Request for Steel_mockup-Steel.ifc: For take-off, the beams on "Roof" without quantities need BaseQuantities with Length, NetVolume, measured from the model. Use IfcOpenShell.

First a look at what the model holds.

```python
import ifcopenshell
import ifcopenshell.util.element
import ifcopenshell.util.unit

model = ifcopenshell.open("Steel_mockup-Steel.ifc")
print(model.schema)
for unit_type in ("LENGTHUNIT", "AREAUNIT", "VOLUMEUNIT"):
    print(unit_type, ifcopenshell.util.unit.calculate_unit_scale(model, unit_type))
storey = next(s for s in model.by_type("IfcBuildingStorey") if s.Name == "Roof")
beams = [e for e in ifcopenshell.util.element.get_decomposition(storey) if e.is_a("IfcBeam")]
for e in sorted(beams, key=lambda e: e.id()):
    print(e.id(), e.is_a(), e.Name, list(ifcopenshell.util.element.get_psets(e, qtos_only=True)), sep=" | ")
```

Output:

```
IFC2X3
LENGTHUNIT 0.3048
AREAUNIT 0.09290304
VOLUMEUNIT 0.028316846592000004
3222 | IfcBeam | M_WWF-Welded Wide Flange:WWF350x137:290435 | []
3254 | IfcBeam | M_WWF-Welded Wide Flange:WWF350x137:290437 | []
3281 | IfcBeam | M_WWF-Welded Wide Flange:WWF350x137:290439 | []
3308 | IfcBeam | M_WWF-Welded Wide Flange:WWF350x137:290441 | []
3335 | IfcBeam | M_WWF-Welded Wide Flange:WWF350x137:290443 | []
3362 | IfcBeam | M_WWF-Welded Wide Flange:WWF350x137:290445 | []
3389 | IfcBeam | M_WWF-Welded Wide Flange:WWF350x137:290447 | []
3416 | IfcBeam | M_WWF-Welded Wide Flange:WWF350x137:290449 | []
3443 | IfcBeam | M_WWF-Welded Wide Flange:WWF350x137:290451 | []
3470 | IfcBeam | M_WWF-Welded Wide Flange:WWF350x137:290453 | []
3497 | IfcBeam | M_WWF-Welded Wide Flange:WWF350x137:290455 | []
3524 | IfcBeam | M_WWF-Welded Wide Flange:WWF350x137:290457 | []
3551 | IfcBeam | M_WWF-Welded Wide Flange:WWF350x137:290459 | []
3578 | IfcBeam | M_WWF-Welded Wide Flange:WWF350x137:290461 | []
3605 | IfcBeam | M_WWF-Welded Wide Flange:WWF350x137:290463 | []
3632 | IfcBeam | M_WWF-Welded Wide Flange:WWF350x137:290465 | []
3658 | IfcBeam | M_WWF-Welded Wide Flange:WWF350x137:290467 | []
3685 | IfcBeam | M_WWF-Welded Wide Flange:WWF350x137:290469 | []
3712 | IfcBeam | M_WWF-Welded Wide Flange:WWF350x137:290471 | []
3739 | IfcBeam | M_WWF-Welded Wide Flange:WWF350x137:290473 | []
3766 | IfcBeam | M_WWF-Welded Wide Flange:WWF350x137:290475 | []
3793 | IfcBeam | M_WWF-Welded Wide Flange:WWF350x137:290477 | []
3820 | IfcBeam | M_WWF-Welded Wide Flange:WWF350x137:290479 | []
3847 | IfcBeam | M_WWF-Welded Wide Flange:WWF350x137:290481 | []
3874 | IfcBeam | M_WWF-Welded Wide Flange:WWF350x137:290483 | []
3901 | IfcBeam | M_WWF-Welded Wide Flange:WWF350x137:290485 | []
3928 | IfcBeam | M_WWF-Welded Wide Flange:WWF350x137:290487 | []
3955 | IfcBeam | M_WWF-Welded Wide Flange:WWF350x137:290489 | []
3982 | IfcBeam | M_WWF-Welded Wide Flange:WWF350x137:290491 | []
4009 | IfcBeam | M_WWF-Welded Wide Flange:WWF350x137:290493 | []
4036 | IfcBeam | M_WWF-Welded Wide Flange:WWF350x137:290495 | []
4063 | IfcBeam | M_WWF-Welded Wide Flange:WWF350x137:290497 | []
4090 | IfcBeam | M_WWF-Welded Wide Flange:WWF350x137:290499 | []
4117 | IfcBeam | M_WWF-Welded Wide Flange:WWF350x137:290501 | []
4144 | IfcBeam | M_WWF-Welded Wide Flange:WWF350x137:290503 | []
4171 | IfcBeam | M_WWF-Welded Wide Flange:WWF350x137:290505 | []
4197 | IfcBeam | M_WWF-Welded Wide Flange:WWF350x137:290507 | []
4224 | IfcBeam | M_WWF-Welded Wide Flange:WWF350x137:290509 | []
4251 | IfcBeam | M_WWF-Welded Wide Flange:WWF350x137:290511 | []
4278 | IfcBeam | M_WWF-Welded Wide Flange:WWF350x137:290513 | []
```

```python
import ifcopenshell
import ifcopenshell.api.pset
import ifcopenshell.geom
import ifcopenshell.util.element
import ifcopenshell.util.shape
import ifcopenshell.util.unit

model = ifcopenshell.open("Steel_mockup-Steel.ifc")
unit_scale = ifcopenshell.util.unit.calculate_unit_scale(model)
volume_scale = ifcopenshell.util.unit.calculate_unit_scale(model, "VOLUMEUNIT")
settings = ifcopenshell.geom.settings()

storey = next(s for s in model.by_type("IfcBuildingStorey") if s.Name == "Roof")
beams = [e for e in ifcopenshell.util.element.get_decomposition(storey) if e.is_a("IfcBeam")]

for e in sorted(beams, key=lambda e: e.id()):
    if ifcopenshell.util.element.get_psets(e, qtos_only=True, should_inherit=False):
        continue
    # Geometry comes back in metres, in the element's own axes.
    shape = ifcopenshell.geom.create_shape(settings, e)
    values = {
        "Length": ifcopenshell.util.shape.get_max_xyz(shape.geometry) / unit_scale,
        "NetVolume": ifcopenshell.util.shape.get_volume(shape.geometry) / volume_scale,
    }
    qto = ifcopenshell.api.pset.add_qto(model, product=e, name="BaseQuantities")
    ifcopenshell.api.pset.edit_qto(model, qto=qto, properties=values)
    print(e.id(), {k: round(v, 3) for k, v in values.items()})

model.write("Steel_mockup-Steel_rev.ifc")
```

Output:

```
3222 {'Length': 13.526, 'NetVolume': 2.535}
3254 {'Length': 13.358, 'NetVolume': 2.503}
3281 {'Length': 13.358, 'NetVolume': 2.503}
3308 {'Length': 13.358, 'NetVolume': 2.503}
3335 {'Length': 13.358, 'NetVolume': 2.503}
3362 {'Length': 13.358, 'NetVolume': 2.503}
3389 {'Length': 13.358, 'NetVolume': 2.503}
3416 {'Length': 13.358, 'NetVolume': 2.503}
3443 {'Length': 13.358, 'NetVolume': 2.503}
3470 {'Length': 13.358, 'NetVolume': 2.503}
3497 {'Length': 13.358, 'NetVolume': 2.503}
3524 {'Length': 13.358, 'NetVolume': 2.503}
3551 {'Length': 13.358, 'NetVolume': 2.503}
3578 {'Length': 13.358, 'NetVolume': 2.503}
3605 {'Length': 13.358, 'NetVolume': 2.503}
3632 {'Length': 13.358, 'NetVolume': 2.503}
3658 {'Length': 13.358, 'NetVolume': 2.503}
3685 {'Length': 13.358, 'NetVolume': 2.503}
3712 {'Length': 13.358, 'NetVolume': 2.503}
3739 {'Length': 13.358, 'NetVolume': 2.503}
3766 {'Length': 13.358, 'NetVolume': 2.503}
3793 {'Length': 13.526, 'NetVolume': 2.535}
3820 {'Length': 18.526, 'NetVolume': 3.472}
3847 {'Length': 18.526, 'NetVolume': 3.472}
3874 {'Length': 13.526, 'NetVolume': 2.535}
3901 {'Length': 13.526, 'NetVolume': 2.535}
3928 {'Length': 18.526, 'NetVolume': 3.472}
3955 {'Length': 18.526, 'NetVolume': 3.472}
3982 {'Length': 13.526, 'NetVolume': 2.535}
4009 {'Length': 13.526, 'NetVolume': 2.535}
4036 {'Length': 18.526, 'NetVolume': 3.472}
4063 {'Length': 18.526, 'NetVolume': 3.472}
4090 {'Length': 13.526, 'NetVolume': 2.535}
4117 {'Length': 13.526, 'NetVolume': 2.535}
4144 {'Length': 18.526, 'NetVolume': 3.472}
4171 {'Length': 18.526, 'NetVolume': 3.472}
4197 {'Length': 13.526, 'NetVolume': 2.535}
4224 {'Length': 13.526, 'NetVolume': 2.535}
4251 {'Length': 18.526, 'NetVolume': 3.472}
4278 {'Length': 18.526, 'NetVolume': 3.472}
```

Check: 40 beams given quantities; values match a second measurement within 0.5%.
